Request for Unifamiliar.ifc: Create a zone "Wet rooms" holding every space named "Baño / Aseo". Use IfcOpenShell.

First a look at what the model holds.

```python
import ifcopenshell

model = ifcopenshell.open("Unifamiliar.ifc")
print(model.schema)
seen = {}
for space in model.by_type("IfcSpace"):
    seen[space.LongName] = seen.get(space.LongName, 0) + 1
for name, count in sorted(seen.items(), key=str):
    print(count, "x", name)
print("zones:", [z.Name for z in model.by_type("IfcZone")][:20])
```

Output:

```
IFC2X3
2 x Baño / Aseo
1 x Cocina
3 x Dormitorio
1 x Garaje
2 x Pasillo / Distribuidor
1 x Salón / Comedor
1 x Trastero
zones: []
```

```python
import ifcopenshell
import ifcopenshell.api.group
import ifcopenshell.api.root

model = ifcopenshell.open("Unifamiliar.ifc")

names = {"Baño / Aseo"}
spaces = [s for s in model.by_type("IfcSpace") if s.LongName in names]

zone = ifcopenshell.api.root.create_entity(model, ifc_class="IfcZone", name="Wet rooms")
ifcopenshell.api.group.assign_group(model, products=spaces, group=zone)
print(len(spaces), "spaces in", zone.Name)

model.write("Unifamiliar_edited.ifc")
```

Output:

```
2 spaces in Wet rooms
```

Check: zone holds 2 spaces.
